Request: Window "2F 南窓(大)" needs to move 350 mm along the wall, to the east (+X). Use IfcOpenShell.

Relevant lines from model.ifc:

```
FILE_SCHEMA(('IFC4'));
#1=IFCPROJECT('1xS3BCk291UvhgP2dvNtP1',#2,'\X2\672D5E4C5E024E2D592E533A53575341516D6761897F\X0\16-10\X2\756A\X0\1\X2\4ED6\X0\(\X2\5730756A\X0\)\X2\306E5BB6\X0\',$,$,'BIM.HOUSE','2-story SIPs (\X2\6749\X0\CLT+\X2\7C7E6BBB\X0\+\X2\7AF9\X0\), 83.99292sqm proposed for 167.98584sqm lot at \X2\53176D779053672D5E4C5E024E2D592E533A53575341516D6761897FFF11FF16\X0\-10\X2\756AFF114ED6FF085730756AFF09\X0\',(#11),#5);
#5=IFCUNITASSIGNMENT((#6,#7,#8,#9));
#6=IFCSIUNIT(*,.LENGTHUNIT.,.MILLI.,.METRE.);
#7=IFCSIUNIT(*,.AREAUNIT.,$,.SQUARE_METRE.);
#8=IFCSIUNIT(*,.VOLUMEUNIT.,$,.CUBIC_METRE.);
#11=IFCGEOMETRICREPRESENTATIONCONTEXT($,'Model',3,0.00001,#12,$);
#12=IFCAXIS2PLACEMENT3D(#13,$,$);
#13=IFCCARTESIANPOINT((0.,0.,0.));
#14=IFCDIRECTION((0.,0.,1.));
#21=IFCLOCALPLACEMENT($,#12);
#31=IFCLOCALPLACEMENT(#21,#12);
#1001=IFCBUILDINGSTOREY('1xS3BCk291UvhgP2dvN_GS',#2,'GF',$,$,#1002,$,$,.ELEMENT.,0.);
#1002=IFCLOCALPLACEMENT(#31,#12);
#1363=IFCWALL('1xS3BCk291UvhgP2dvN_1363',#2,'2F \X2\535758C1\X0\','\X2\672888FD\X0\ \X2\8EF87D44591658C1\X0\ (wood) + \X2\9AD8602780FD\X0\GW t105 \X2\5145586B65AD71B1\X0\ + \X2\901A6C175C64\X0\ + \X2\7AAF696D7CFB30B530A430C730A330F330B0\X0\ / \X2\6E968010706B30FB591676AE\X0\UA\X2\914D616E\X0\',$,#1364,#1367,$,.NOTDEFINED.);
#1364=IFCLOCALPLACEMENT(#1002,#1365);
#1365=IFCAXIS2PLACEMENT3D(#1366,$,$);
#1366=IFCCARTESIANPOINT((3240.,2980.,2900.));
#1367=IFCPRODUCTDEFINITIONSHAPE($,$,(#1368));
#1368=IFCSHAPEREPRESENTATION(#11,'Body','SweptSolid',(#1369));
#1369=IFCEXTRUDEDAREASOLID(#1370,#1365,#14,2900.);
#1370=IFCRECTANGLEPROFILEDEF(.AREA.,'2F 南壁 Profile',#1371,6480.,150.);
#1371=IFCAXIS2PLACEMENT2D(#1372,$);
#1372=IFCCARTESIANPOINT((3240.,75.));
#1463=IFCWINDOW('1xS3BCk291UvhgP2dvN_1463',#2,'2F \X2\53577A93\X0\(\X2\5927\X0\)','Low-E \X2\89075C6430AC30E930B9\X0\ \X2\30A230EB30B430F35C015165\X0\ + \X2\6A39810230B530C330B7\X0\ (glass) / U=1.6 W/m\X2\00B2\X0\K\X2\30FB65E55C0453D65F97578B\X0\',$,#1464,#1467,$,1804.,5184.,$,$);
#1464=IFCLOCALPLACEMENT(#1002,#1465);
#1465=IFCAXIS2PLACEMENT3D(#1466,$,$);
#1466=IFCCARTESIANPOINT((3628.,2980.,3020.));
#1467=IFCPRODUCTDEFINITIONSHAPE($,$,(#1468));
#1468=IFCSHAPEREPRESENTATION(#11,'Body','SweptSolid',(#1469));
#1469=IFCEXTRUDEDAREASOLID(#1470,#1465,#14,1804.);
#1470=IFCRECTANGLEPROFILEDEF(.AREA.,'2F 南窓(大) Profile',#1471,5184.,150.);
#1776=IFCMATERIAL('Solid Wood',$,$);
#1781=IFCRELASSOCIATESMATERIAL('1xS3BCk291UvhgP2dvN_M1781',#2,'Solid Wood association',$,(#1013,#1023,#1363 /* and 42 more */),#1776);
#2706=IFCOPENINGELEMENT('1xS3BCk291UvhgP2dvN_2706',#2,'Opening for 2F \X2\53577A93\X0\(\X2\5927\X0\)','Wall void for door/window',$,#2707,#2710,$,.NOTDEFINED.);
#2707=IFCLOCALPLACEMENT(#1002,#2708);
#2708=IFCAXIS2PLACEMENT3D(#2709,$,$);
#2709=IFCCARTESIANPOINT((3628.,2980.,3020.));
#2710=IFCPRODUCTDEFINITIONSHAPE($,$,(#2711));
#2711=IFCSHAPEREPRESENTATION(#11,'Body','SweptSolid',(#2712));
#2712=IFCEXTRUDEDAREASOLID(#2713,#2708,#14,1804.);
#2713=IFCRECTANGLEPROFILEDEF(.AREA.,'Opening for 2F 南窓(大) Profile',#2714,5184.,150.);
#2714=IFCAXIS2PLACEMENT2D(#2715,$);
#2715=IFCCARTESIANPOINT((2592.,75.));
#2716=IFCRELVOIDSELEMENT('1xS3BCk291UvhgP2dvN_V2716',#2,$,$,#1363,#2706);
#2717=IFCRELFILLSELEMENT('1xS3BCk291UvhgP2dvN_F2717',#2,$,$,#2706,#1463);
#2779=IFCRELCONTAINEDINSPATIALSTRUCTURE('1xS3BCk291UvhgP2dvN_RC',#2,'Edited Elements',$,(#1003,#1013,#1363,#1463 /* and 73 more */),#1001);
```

```python
import ifcopenshell
import ifcopenshell.api.geometry
import ifcopenshell.util.placement
import ifcopenshell.util.unit

model = ifcopenshell.open("model.ifc")
unit_scale = ifcopenshell.util.unit.calculate_unit_scale(model)

window = model.by_guid("1xS3BCk291UvhgP2dvN_1463")
opening = window.FillsVoids[0].RelatingOpeningElement
wall = opening.VoidsElements[0].RelatingBuildingElement

wall_matrix = ifcopenshell.util.placement.get_local_placement(wall.ObjectPlacement)
shift = wall_matrix[:3, 0] * 0.35 / unit_scale
before = ifcopenshell.util.placement.get_local_placement(window.ObjectPlacement)[:3, 3].copy()

# The window is not placed relative to its opening, so move both.
for product in (opening, window):
    matrix = ifcopenshell.util.placement.get_local_placement(product.ObjectPlacement)
    matrix[:3, 3] += shift
    ifcopenshell.api.geometry.edit_object_placement(model, product=product, matrix=matrix, is_si=False)

after = ifcopenshell.util.placement.get_local_placement(window.ObjectPlacement)[:3, 3]
print("window moved by", (after - before).round(3) + 0.0)

model.write("model_updated.ifc")
```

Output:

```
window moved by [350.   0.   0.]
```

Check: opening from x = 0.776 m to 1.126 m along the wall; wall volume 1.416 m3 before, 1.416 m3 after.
